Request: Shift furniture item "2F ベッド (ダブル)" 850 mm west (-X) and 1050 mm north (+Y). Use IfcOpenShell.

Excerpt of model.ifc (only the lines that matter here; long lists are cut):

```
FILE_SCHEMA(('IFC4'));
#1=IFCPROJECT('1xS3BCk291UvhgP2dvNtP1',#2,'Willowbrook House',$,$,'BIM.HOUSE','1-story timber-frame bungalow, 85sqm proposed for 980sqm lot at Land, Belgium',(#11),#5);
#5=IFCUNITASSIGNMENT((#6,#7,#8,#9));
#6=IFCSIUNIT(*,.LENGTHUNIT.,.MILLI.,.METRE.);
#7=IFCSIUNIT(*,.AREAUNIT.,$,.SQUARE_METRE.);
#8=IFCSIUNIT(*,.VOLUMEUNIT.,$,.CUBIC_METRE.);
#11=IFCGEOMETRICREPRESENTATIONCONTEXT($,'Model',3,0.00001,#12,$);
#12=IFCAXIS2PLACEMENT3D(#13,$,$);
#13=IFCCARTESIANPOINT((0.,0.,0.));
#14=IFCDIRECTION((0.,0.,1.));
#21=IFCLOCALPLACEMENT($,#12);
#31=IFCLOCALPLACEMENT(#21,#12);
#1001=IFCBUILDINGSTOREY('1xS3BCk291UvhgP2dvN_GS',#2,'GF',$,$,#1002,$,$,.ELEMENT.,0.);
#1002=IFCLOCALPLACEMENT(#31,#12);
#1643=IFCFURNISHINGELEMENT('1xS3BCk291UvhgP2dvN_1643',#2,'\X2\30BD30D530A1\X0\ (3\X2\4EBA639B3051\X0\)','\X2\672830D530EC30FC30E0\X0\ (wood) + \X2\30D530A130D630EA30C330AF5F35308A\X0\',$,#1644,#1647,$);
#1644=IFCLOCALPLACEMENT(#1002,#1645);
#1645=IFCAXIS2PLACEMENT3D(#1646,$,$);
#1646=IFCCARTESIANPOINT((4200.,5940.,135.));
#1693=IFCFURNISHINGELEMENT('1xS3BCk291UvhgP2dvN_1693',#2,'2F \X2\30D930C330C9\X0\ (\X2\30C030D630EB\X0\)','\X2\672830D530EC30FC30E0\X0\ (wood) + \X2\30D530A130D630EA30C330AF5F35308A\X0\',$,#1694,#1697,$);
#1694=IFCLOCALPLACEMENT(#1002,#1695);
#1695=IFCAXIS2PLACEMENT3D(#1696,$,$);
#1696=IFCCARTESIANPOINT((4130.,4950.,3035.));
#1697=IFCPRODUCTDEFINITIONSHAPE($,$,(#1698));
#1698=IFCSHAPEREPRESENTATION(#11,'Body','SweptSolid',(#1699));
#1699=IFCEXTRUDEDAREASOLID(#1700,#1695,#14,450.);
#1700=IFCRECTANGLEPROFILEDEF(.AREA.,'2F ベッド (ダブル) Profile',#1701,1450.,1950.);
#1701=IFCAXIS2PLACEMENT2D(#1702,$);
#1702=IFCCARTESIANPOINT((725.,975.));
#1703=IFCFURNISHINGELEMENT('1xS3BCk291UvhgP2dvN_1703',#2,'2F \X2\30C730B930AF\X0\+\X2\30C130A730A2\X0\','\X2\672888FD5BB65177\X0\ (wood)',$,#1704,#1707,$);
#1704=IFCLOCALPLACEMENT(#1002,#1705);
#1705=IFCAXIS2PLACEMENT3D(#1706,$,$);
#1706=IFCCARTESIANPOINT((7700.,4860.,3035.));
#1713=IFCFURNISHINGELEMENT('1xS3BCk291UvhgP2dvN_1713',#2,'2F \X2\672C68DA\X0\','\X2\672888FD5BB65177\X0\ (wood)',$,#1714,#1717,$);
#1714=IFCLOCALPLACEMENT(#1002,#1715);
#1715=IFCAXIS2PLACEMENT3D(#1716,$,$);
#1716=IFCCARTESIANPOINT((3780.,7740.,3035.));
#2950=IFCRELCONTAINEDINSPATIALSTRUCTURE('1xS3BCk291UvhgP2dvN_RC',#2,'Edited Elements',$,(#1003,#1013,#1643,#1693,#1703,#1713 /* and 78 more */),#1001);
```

```python
import ifcopenshell
import ifcopenshell.api.geometry
import ifcopenshell.util.placement
import ifcopenshell.util.unit

model = ifcopenshell.open("model.ifc")
unit_scale = ifcopenshell.util.unit.calculate_unit_scale(model)

item = model.by_guid("1xS3BCk291UvhgP2dvN_1693")
matrix = ifcopenshell.util.placement.get_local_placement(item.ObjectPlacement)
matrix[0, 3] -= 0.85 / unit_scale
matrix[1, 3] += 1.05 / unit_scale
ifcopenshell.api.geometry.edit_object_placement(model, product=item, matrix=matrix, is_si=False)

print(ifcopenshell.util.placement.get_local_placement(item.ObjectPlacement).round(3) + 0.0)

model.write("model-out.ifc")
```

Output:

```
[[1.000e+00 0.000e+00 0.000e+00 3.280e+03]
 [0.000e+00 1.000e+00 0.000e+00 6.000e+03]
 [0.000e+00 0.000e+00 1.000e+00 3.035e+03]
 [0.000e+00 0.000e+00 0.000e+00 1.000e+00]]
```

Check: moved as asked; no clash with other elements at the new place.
